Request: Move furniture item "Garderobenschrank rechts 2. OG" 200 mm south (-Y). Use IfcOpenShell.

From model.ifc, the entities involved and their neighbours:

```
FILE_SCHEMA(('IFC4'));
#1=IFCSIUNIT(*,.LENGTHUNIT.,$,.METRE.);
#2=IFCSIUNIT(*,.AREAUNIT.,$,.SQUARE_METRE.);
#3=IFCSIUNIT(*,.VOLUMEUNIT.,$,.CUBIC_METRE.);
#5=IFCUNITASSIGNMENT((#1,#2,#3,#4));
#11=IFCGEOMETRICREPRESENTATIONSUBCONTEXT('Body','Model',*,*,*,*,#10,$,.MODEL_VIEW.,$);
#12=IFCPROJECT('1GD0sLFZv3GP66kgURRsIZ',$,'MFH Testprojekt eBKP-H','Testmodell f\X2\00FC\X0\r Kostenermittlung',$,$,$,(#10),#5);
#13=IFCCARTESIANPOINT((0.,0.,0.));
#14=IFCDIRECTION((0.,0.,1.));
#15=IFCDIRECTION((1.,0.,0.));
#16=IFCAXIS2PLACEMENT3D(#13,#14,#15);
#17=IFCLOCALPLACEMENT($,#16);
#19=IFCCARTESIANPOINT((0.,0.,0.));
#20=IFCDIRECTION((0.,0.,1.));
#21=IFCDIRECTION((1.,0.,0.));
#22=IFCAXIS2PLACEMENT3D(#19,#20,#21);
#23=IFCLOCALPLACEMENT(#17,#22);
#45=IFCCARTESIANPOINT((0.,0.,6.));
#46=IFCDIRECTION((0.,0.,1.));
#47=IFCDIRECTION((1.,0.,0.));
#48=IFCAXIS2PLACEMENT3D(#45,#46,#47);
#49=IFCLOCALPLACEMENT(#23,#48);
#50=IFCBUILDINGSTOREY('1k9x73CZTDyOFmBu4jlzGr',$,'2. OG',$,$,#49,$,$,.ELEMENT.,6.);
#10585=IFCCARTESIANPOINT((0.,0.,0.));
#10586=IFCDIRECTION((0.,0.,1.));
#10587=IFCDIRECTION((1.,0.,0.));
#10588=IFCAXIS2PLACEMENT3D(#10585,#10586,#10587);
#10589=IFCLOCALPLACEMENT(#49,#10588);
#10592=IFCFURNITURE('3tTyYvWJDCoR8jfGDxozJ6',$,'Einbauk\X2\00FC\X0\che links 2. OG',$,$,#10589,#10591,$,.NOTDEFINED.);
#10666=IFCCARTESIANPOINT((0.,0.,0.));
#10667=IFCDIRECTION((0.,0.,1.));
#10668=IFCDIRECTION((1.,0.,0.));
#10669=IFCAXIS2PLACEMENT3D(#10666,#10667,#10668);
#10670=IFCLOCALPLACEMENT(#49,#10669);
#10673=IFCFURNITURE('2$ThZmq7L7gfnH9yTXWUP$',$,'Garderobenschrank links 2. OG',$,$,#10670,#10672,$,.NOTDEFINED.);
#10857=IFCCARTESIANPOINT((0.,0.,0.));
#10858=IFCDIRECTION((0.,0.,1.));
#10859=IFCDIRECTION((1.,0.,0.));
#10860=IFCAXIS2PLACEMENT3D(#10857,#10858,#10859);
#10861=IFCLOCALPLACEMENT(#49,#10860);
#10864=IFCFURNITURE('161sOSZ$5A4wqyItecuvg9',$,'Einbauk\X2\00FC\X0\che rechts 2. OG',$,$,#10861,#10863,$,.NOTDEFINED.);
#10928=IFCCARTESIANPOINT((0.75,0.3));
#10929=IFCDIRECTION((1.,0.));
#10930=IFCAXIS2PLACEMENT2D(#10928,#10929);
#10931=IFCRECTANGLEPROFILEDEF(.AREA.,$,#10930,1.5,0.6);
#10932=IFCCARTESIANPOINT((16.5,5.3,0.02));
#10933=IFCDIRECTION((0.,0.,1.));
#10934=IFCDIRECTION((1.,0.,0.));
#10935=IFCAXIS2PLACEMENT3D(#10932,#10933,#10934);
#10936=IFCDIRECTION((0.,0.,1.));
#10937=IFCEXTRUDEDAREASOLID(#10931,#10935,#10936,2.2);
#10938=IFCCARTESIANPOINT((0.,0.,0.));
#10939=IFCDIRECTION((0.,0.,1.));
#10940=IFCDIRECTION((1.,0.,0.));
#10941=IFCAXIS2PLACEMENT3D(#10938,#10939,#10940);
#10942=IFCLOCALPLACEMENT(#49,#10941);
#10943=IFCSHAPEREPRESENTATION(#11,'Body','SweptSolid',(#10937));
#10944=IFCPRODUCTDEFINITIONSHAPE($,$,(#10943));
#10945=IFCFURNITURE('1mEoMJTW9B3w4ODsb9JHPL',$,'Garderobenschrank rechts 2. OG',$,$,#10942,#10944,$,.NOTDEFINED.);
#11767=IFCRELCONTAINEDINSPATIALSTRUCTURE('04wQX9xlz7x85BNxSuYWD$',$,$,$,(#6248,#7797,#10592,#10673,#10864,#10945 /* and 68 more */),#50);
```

```python
import ifcopenshell
import ifcopenshell.api.geometry
import ifcopenshell.util.placement
import ifcopenshell.util.unit

model = ifcopenshell.open("model.ifc")
unit_scale = ifcopenshell.util.unit.calculate_unit_scale(model)

item = model.by_id(10945)
matrix = ifcopenshell.util.placement.get_local_placement(item.ObjectPlacement)
matrix[1, 3] -= 0.2 / unit_scale
ifcopenshell.api.geometry.edit_object_placement(model, product=item, matrix=matrix, is_si=False)

print(ifcopenshell.util.placement.get_local_placement(item.ObjectPlacement).round(3) + 0.0)

model.write("model_v2.ifc")
```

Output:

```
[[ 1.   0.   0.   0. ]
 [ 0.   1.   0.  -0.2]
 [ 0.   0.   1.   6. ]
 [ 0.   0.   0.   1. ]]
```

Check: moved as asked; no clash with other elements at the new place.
